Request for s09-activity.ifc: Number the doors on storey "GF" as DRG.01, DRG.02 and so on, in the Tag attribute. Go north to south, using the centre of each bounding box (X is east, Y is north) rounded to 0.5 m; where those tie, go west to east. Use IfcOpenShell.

First a look at what the model holds.

```python
import ifcopenshell
import ifcopenshell.util.element
import ifcopenshell.util.placement

model = ifcopenshell.open("s09-activity.ifc")
print(model.schema)
storey = next(s for s in model.by_type("IfcBuildingStorey") if s.Name == "GF")
doors = [e for e in ifcopenshell.util.element.get_decomposition(storey) if e.is_a("IfcDoor")]
for e in sorted(doors, key=lambda e: e.id()):
    origin = ifcopenshell.util.placement.get_local_placement(e.ObjectPlacement)[:3, 3]
    print(e.id(), e.Tag, e.Name, origin.round(2) + 0.0, sep=" | ")
```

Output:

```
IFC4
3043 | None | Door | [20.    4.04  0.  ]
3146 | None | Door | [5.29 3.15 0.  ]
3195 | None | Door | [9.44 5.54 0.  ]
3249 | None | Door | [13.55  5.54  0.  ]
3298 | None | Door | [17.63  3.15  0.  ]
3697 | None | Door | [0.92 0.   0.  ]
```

```python
import ifcopenshell
import ifcopenshell.geom
import ifcopenshell.util.element
import ifcopenshell.util.shape

model = ifcopenshell.open("s09-activity.ifc")
settings = ifcopenshell.geom.settings()
settings.set("use-world-coords", True)


def centre(element):
    shape = ifcopenshell.geom.create_shape(settings, element)
    return ifcopenshell.util.shape.get_bbox_centroid(shape.geometry)


storey = next(s for s in model.by_type("IfcBuildingStorey") if s.Name == "GF")
doors = [e for e in ifcopenshell.util.element.get_decomposition(storey) if e.is_a("IfcDoor")]

# Insertion points can sit at a corner or the storey origin, so sort by the geometry (in metres).
centres = {e: centre(e) for e in doors}
doors.sort(key=lambda e: (-round(centres[e][1] / 0.5), centres[e][0]))

for i, e in enumerate(doors, start=1):
    number = f"DRG.{i:02d}"
    e.Tag = number
    print(e.id(), number)

model.write("s09-activity_v2.ifc")
```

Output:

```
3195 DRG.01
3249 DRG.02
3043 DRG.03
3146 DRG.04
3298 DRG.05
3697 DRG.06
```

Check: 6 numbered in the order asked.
